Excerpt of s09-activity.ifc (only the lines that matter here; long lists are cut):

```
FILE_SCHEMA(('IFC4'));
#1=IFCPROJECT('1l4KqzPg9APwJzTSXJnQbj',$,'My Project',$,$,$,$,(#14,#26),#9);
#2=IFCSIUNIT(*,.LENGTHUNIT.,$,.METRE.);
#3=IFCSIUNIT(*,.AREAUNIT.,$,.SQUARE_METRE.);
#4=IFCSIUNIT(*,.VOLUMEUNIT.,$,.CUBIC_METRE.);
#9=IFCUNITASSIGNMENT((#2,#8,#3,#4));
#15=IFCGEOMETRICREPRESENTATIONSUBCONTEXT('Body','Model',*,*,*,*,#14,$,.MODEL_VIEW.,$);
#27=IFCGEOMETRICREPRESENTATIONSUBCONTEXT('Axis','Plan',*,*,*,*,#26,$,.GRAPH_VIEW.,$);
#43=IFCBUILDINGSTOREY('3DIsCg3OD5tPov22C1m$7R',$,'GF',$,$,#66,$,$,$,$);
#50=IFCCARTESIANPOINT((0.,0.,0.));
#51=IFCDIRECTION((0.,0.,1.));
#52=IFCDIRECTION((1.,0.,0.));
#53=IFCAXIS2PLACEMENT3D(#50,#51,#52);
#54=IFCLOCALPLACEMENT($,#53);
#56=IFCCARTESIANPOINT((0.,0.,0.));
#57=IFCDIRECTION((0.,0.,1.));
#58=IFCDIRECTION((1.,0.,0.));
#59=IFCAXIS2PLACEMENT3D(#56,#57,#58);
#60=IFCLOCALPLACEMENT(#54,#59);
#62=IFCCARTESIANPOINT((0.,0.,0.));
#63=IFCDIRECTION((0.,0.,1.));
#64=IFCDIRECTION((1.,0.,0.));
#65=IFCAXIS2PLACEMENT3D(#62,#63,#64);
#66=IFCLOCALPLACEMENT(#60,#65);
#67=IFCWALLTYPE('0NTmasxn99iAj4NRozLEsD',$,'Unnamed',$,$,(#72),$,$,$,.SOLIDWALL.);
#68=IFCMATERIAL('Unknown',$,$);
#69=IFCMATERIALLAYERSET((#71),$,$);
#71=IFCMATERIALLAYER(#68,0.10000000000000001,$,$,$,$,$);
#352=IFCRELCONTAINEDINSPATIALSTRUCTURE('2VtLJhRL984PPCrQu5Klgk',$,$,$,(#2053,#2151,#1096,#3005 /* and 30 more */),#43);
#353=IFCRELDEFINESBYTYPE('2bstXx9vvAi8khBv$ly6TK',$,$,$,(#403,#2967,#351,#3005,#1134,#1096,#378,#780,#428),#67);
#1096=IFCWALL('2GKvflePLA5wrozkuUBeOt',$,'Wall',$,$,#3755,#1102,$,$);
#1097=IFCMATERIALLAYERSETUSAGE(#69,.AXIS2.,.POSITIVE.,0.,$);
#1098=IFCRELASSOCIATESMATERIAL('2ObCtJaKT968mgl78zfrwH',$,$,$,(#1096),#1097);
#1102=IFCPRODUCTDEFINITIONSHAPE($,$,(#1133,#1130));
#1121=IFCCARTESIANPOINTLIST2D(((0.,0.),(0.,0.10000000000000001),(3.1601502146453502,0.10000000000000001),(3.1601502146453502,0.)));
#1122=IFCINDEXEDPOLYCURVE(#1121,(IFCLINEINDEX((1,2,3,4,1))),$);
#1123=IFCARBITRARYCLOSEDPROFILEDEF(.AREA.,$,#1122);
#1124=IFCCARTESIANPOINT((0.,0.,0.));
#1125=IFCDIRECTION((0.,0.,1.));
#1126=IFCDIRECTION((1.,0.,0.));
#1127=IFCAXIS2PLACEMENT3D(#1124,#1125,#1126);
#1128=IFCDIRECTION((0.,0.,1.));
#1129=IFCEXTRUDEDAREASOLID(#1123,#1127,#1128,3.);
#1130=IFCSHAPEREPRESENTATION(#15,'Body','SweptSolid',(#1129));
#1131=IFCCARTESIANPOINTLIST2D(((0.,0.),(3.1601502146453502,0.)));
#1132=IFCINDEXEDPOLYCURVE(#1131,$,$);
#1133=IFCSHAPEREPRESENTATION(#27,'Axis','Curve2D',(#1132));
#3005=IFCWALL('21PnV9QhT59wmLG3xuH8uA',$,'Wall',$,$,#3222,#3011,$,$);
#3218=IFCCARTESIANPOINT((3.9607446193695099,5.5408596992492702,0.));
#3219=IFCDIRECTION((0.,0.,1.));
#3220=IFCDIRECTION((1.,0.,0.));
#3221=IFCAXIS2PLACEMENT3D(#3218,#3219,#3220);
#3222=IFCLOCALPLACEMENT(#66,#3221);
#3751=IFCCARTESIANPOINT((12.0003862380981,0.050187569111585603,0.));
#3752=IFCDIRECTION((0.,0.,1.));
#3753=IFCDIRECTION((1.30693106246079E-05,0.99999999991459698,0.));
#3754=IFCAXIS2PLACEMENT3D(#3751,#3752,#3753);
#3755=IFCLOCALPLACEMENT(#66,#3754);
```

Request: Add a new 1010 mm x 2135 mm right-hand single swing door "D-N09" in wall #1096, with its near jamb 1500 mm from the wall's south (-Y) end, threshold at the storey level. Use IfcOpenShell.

```python
import numpy as np
import ifcopenshell
import ifcopenshell.api.feature
import ifcopenshell.api.geometry
import ifcopenshell.api.root
import ifcopenshell.api.spatial
import ifcopenshell.geom
import ifcopenshell.util.element
import ifcopenshell.util.placement
import ifcopenshell.util.representation
import ifcopenshell.util.shape
import ifcopenshell.util.unit

model = ifcopenshell.open("s09-activity.ifc")
unit_scale = ifcopenshell.util.unit.calculate_unit_scale(model)
settings = ifcopenshell.geom.settings()


def volume(element):
    """Net volume in cubic metres, openings subtracted."""
    shape = ifcopenshell.geom.create_shape(settings, element)
    return ifcopenshell.util.shape.get_volume(shape.geometry)


wall = model.by_guid("2GKvflePLA5wrozkuUBeOt")
storey = ifcopenshell.util.element.get_container(wall, ifc_class="IfcBuildingStorey")
context = ifcopenshell.util.representation.get_context(model, "Model", "Body", "MODEL_VIEW")
before = volume(wall)

width, height, from_end, sill = 1.01, 2.135, 1.5, 0.0  # metres

# The wall runs along its own X axis, and the end named is its -X end.
wall_shape = ifcopenshell.geom.create_shape(settings, wall)
x, y, z = ifcopenshell.util.shape.get_vertices(wall_shape.geometry).T
start = x.min() + from_end
face, thickness = float(y.min()), float(y.max() - y.min())
wall_matrix = ifcopenshell.util.placement.get_local_placement(wall.ObjectPlacement)
level = ifcopenshell.util.placement.get_local_placement(storey.ObjectPlacement)[2, 3]


def in_wall(x, y):
    """Placement at x, y metres in the wall's axes, at sill height."""
    matrix = wall_matrix.copy()
    matrix[:, 3] = wall_matrix @ np.array([x / unit_scale, y / unit_scale, 0.0, 1.0])
    matrix[2, 3] = level + sill / unit_scale
    return matrix


# Opening: a box that overshoots both wall faces by 50 mm.
opening = ifcopenshell.api.root.create_entity(model, ifc_class="IfcOpeningElement", predefined_type="OPENING")
box = ifcopenshell.api.geometry.add_wall_representation(
    model, context=context, length=width, height=height, thickness=thickness + 0.1
)
ifcopenshell.api.geometry.assign_representation(model, product=opening, representation=box)
ifcopenshell.api.geometry.edit_object_placement(model, product=opening, matrix=in_wall(start, face - 0.05), is_si=False)
ifcopenshell.api.feature.add_feature(model, feature=opening, element=wall)

door = ifcopenshell.api.root.create_entity(model, ifc_class="IfcDoor", name="D-N09", predefined_type="DOOR")
door.OverallWidth, door.OverallHeight = width / unit_scale, height / unit_scale
door.OperationType = "SINGLE_SWING_RIGHT"
body = ifcopenshell.api.geometry.add_door_representation(
    model,
    context=context,
    overall_width=door.OverallWidth,
    overall_height=door.OverallHeight,
    operation_type="SINGLE_SWING_RIGHT",
    lining_properties={"LiningDepth": thickness / unit_scale, "ThresholdDepth": thickness / unit_scale},
)
ifcopenshell.api.geometry.assign_representation(model, product=door, representation=body)
ifcopenshell.api.spatial.assign_container(model, products=[door], relating_structure=storey)
ifcopenshell.api.feature.add_filling(model, opening=opening, element=door)

# The lining spans the wall, so the door starts at the wall face.
ifcopenshell.api.geometry.edit_object_placement(model, product=door, matrix=in_wall(start, face), is_si=False)

after = volume(wall)

print(f"wall volume {before:.3f} -> {after:.3f} m3")

model.write("s09-activity_rev.ifc")
```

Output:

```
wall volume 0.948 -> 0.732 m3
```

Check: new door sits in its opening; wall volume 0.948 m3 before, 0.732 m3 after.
